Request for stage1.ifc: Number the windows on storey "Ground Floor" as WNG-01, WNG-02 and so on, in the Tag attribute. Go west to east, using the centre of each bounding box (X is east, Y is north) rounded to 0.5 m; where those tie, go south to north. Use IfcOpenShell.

First a look at what the model holds.

```python
import ifcopenshell
import ifcopenshell.util.element
import ifcopenshell.util.placement

model = ifcopenshell.open("stage1.ifc")
print(model.schema)
storey = next(s for s in model.by_type("IfcBuildingStorey") if s.Name == "Ground Floor")
windows = [e for e in ifcopenshell.util.element.get_decomposition(storey) if e.is_a("IfcWindow")]
for e in sorted(windows, key=lambda e: e.id()):
    origin = ifcopenshell.util.placement.get_local_placement(e.ObjectPlacement)[:3, 3]
    print(e.id(), e.Tag, e.Name, origin.round(2) + 0.0, sep=" | ")
```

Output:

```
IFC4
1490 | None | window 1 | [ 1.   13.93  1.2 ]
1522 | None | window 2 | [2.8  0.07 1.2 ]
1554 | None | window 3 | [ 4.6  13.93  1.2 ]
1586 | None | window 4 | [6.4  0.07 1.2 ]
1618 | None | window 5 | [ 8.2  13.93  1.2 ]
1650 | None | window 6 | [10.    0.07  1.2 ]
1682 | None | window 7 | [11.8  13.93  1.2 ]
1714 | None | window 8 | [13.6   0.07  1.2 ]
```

```python
import ifcopenshell
import ifcopenshell.geom
import ifcopenshell.util.element
import ifcopenshell.util.shape

model = ifcopenshell.open("stage1.ifc")
settings = ifcopenshell.geom.settings()
settings.set("use-world-coords", True)


def centre(element):
    shape = ifcopenshell.geom.create_shape(settings, element)
    return ifcopenshell.util.shape.get_bbox_centroid(shape.geometry)


storey = next(s for s in model.by_type("IfcBuildingStorey") if s.Name == "Ground Floor")
windows = [e for e in ifcopenshell.util.element.get_decomposition(storey) if e.is_a("IfcWindow")]

# Insertion points can sit at a corner or the storey origin, so sort by the geometry (in metres).
centres = {e: centre(e) for e in windows}
windows.sort(key=lambda e: (round(centres[e][0] / 0.5), centres[e][1]))

for i, e in enumerate(windows, start=1):
    number = f"WNG-{i:02d}"
    e.Tag = number
    print(e.id(), number)

model.write("stage1-out.ifc")
```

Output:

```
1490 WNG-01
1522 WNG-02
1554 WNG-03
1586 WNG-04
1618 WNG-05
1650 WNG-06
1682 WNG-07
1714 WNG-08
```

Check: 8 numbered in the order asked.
